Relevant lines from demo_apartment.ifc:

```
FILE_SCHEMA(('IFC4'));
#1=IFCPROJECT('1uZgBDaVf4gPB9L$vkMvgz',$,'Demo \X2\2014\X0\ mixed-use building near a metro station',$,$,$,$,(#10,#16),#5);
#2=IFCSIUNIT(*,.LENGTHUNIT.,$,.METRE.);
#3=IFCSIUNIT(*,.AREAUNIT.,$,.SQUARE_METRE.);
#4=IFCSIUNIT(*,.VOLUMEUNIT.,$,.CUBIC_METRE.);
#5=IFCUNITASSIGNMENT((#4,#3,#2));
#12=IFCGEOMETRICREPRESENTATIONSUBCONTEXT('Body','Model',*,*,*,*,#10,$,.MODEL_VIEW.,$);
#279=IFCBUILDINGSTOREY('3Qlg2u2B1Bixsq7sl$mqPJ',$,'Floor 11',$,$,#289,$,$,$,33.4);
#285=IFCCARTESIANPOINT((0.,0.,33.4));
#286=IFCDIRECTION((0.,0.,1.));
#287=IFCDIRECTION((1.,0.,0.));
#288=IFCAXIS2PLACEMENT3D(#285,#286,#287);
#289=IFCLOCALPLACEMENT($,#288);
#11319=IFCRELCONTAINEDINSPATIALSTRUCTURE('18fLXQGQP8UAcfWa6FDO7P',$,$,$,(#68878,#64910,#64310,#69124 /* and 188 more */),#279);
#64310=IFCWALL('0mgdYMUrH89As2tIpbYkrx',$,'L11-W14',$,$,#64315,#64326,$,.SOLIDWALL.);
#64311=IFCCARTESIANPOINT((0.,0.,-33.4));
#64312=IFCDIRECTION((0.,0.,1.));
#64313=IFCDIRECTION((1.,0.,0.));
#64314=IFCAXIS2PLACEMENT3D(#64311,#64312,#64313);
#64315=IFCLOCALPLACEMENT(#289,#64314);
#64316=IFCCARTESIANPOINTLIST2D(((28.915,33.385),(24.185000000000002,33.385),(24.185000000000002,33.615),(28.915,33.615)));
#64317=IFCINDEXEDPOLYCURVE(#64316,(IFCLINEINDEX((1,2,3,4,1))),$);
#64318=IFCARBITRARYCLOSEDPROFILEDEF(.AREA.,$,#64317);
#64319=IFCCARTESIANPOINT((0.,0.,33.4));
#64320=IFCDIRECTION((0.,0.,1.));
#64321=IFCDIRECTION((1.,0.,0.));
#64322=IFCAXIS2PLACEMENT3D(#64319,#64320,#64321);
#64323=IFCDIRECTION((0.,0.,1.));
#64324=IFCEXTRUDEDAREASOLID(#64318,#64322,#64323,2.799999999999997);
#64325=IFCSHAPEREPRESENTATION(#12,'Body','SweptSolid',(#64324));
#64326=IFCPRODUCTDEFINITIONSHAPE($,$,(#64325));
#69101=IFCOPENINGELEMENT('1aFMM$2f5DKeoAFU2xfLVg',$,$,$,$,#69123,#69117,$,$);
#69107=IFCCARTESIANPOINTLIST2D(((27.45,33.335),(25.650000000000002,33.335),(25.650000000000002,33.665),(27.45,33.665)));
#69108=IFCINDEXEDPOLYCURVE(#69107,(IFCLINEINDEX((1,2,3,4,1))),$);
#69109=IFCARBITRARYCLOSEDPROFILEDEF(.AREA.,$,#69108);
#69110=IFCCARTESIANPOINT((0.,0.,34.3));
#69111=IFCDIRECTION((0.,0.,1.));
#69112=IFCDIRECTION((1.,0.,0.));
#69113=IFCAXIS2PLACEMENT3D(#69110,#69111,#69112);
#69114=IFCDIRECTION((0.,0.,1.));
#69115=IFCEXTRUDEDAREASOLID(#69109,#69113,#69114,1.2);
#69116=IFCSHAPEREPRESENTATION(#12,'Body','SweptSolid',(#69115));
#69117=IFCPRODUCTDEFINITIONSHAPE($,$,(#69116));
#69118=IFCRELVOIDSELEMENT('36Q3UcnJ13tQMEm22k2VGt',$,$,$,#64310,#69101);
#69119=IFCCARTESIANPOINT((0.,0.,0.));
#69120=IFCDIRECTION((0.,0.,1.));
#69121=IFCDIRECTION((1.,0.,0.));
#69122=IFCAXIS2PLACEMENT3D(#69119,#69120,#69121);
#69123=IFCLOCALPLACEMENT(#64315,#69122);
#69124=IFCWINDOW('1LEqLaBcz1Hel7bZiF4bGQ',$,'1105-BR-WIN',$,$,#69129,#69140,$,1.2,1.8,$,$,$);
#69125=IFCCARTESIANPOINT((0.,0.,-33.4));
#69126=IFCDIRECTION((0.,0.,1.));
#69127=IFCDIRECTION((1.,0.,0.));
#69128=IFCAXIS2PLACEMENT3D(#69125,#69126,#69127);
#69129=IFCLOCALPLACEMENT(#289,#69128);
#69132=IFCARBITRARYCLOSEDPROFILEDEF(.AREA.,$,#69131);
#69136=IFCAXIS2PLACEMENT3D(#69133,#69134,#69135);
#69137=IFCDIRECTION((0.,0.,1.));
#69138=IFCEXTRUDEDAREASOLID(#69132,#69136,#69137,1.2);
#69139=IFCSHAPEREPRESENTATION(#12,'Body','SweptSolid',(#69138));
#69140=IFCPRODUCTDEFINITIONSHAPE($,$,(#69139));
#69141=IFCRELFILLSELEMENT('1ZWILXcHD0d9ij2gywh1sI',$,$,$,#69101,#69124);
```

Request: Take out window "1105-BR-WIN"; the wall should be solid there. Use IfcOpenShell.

```python
import ifcopenshell
import ifcopenshell.api.feature
import ifcopenshell.api.root
import ifcopenshell.geom
import ifcopenshell.util.shape

model = ifcopenshell.open("demo_apartment.ifc")
settings = ifcopenshell.geom.settings()


def volume(element):
    """Net volume in cubic metres, openings subtracted."""
    shape = ifcopenshell.geom.create_shape(settings, element)
    return ifcopenshell.util.shape.get_volume(shape.geometry)


window = model.by_id(69124)
opening = window.FillsVoids[0].RelatingOpeningElement
wall = opening.VoidsElements[0].RelatingBuildingElement
before = volume(wall)

ifcopenshell.api.root.remove_product(model, product=window)
ifcopenshell.api.feature.remove_feature(model, feature=opening)

after = volume(wall)

print(f"wall volume {before:.3f} -> {after:.3f} m3")

model.write("demo_apartment_rev.ifc")
```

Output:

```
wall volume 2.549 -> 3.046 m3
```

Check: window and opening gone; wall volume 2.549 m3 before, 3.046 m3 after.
